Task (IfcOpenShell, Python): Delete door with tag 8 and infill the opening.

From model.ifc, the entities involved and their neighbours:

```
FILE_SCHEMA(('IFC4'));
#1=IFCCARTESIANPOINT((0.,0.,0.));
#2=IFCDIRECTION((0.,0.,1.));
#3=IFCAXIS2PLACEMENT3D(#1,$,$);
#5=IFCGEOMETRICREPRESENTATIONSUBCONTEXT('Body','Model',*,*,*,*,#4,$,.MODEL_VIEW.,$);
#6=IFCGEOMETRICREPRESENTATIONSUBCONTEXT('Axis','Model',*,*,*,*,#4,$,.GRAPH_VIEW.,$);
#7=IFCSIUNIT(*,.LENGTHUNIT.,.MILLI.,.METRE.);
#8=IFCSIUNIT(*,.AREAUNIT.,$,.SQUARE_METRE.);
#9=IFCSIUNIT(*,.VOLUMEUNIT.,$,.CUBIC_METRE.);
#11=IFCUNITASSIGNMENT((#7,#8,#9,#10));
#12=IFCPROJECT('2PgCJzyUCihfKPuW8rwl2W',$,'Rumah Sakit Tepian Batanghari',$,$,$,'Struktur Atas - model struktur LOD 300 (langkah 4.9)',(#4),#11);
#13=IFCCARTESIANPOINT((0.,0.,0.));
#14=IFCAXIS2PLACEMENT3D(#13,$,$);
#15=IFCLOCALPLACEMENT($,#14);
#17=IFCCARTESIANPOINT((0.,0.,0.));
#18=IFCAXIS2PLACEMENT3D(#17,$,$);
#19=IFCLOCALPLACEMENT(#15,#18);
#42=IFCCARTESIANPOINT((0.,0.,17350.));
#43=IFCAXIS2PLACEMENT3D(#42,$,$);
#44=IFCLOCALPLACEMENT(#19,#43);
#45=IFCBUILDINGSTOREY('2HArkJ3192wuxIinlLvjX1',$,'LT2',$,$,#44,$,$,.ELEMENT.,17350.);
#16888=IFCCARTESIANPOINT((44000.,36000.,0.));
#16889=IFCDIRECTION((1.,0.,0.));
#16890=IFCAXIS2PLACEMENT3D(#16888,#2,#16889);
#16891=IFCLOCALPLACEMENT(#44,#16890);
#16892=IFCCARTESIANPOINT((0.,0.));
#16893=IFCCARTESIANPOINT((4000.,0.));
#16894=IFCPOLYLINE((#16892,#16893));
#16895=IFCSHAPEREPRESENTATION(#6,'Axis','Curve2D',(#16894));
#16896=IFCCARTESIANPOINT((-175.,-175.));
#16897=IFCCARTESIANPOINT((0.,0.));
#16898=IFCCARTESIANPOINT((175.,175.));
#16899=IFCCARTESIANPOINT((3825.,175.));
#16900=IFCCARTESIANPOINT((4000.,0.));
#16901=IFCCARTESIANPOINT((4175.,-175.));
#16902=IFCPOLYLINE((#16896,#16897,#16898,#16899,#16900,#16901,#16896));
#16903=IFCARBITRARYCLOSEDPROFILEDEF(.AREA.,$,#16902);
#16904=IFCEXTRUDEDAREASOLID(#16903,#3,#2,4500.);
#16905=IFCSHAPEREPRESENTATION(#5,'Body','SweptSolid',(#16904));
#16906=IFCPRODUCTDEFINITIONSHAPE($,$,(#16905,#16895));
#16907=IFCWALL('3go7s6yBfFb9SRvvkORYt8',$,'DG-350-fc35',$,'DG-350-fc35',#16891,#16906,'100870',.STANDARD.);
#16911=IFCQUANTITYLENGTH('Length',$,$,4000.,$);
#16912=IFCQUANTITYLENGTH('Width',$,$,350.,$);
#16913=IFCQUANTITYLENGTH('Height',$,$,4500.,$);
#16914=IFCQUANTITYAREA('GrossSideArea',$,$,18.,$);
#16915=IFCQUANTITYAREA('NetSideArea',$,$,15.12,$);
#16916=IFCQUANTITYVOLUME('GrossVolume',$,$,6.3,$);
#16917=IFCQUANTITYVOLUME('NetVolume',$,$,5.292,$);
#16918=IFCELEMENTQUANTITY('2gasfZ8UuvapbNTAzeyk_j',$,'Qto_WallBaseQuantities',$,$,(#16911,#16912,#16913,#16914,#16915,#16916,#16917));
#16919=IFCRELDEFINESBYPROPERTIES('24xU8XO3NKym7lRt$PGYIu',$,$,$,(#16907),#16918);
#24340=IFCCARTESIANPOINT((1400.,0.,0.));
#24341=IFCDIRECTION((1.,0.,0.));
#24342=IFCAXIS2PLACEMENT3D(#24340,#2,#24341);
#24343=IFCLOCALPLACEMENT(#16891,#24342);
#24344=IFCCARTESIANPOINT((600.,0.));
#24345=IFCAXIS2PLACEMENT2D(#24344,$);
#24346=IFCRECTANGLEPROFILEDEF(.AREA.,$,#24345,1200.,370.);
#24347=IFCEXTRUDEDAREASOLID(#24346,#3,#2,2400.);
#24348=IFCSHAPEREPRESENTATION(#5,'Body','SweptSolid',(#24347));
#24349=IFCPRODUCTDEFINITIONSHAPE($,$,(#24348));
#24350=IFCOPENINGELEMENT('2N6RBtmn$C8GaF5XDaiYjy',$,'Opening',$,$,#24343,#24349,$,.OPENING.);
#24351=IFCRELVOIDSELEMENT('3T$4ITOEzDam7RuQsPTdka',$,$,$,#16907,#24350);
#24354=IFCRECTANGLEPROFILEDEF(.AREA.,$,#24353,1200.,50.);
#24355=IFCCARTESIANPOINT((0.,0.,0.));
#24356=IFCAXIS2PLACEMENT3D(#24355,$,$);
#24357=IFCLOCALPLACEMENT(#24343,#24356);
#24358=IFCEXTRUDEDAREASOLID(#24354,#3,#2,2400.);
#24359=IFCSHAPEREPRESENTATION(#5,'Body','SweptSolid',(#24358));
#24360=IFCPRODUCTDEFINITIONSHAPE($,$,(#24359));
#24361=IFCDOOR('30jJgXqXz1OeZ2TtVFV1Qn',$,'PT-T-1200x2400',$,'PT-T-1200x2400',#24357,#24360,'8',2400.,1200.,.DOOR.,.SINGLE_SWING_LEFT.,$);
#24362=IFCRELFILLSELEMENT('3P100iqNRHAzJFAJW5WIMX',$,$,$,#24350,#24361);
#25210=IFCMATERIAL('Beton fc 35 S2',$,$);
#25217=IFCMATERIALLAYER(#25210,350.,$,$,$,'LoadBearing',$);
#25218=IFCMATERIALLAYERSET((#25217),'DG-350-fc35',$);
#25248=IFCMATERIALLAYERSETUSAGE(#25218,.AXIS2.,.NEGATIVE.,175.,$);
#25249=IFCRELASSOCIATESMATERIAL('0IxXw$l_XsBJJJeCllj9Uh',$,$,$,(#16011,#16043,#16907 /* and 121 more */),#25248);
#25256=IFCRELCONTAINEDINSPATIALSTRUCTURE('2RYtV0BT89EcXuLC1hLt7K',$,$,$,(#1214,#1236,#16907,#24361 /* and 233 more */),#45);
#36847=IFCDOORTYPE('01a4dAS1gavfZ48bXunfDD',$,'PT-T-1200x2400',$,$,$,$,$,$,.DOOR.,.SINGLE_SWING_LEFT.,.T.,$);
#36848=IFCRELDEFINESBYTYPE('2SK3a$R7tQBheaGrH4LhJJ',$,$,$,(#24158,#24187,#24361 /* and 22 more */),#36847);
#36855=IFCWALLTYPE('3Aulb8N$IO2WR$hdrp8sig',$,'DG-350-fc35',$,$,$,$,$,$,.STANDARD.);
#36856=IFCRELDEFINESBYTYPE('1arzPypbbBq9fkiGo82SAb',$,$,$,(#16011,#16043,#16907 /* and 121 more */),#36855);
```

```python
import ifcopenshell
import ifcopenshell.api.feature
import ifcopenshell.api.pset
import ifcopenshell.api.root
import ifcopenshell.geom
import ifcopenshell.util.element
import ifcopenshell.util.shape
import ifcopenshell.util.unit

model = ifcopenshell.open("model.ifc")
area_scale = ifcopenshell.util.unit.calculate_unit_scale(model, "AREAUNIT")
volume_scale = ifcopenshell.util.unit.calculate_unit_scale(model, "VOLUMEUNIT")
settings = ifcopenshell.geom.settings()


def volume(element):
    """Net volume in cubic metres, openings subtracted."""
    shape = ifcopenshell.geom.create_shape(settings, element)
    return ifcopenshell.util.shape.get_volume(shape.geometry)


door = model.by_guid("30jJgXqXz1OeZ2TtVFV1Qn")
opening = door.FillsVoids[0].RelatingOpeningElement
wall = opening.VoidsElements[0].RelatingBuildingElement
before = volume(wall)

ifcopenshell.api.root.remove_product(model, product=door)
ifcopenshell.api.feature.remove_feature(model, feature=opening)

after = volume(wall)
thickness = 0.35  # wall thickness in metres

# Update the wall's stored quantities.
qto = model.by_id(ifcopenshell.util.element.get_pset(wall, "Qto_WallBaseQuantities", should_inherit=False)["id"])
ifcopenshell.api.pset.edit_qto(model, qto=qto, properties={
    "NetSideArea": after / thickness / area_scale,
    "NetVolume": after / volume_scale,
})

print(f"wall volume {before:.3f} -> {after:.3f} m3")

model.write("model_edited.ifc")
```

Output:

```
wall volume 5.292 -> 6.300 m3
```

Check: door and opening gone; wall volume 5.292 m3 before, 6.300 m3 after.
